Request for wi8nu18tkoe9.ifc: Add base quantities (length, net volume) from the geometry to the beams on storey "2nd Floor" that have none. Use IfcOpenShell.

First a look at what the model holds.

```python
import ifcopenshell
import ifcopenshell.util.element
import ifcopenshell.util.unit

model = ifcopenshell.open("wi8nu18tkoe9.ifc")
print(model.schema)
for unit_type in ("LENGTHUNIT", "AREAUNIT", "VOLUMEUNIT"):
    print(unit_type, ifcopenshell.util.unit.calculate_unit_scale(model, unit_type))
storey = next(s for s in model.by_type("IfcBuildingStorey") if s.Name == "2nd Floor")
beams = [e for e in ifcopenshell.util.element.get_decomposition(storey) if e.is_a("IfcBeam")]
for e in sorted(beams, key=lambda e: e.id()):
    print(e.id(), e.is_a(), e.Name, list(ifcopenshell.util.element.get_psets(e, qtos_only=True)), sep=" | ")
```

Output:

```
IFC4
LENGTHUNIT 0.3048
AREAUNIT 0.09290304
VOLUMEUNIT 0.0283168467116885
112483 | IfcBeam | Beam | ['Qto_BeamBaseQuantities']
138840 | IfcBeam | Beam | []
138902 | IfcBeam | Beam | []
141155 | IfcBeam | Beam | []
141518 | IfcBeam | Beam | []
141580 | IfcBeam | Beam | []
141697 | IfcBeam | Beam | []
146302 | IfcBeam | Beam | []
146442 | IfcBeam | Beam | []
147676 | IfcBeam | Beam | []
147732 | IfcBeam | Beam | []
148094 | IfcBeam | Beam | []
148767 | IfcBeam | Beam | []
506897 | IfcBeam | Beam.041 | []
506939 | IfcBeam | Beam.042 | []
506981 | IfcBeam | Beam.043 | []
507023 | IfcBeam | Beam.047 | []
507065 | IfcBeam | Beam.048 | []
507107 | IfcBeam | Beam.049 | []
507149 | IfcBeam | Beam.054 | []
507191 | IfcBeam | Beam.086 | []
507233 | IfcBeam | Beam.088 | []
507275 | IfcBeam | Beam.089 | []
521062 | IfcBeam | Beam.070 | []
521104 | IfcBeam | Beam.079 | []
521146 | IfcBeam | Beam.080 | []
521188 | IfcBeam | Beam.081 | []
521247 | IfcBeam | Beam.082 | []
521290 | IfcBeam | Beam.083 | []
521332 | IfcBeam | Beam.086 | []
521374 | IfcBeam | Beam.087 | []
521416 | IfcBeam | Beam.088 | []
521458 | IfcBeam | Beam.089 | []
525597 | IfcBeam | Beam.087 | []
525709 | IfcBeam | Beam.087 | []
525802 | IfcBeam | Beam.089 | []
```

```python
import ifcopenshell
import ifcopenshell.api.pset
import ifcopenshell.geom
import ifcopenshell.util.element
import ifcopenshell.util.shape
import ifcopenshell.util.unit

model = ifcopenshell.open("wi8nu18tkoe9.ifc")
unit_scale = ifcopenshell.util.unit.calculate_unit_scale(model)
volume_scale = ifcopenshell.util.unit.calculate_unit_scale(model, "VOLUMEUNIT")
settings = ifcopenshell.geom.settings()

storey = next(s for s in model.by_type("IfcBuildingStorey") if s.Name == "2nd Floor")
beams = [e for e in ifcopenshell.util.element.get_decomposition(storey) if e.is_a("IfcBeam")]

for e in sorted(beams, key=lambda e: e.id()):
    if ifcopenshell.util.element.get_psets(e, qtos_only=True, should_inherit=False):
        continue
    # Geometry comes back in metres, in the element's own axes.
    shape = ifcopenshell.geom.create_shape(settings, e)
    values = {
        "Length": ifcopenshell.util.shape.get_max_xyz(shape.geometry) / unit_scale,
        "NetVolume": ifcopenshell.util.shape.get_volume(shape.geometry) / volume_scale,
    }
    qto = ifcopenshell.api.pset.add_qto(model, product=e, name="Qto_BeamBaseQuantities")
    ifcopenshell.api.pset.edit_qto(model, qto=qto, properties=values)
    print(e.id(), {k: round(v, 3) for k, v in values.items()})

model.write("wi8nu18tkoe9_edited.ifc")
```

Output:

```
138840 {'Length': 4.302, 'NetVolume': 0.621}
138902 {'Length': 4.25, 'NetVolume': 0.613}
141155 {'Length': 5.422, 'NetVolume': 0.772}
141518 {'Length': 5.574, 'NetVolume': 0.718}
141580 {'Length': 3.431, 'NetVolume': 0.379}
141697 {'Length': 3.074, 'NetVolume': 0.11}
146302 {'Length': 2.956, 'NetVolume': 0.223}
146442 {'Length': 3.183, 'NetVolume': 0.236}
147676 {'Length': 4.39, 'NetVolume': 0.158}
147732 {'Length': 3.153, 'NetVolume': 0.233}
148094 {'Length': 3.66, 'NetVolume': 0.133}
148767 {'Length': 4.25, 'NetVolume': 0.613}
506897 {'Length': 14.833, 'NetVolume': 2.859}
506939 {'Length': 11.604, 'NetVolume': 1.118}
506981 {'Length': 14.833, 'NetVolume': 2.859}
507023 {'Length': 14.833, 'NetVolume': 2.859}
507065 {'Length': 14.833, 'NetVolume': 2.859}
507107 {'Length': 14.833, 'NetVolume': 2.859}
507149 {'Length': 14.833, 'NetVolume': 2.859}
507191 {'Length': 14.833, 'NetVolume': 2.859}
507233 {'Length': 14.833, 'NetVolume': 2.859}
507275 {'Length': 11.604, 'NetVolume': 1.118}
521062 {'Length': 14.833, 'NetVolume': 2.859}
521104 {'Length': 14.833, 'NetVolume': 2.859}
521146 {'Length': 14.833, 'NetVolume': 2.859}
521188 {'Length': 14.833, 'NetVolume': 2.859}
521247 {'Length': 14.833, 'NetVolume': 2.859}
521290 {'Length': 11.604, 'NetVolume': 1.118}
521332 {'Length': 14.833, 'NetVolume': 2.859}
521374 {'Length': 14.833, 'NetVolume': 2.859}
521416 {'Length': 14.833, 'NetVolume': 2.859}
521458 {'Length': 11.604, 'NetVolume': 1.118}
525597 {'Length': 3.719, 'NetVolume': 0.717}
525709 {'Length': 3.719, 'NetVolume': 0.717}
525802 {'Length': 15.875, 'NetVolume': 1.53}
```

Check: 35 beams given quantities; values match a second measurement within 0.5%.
